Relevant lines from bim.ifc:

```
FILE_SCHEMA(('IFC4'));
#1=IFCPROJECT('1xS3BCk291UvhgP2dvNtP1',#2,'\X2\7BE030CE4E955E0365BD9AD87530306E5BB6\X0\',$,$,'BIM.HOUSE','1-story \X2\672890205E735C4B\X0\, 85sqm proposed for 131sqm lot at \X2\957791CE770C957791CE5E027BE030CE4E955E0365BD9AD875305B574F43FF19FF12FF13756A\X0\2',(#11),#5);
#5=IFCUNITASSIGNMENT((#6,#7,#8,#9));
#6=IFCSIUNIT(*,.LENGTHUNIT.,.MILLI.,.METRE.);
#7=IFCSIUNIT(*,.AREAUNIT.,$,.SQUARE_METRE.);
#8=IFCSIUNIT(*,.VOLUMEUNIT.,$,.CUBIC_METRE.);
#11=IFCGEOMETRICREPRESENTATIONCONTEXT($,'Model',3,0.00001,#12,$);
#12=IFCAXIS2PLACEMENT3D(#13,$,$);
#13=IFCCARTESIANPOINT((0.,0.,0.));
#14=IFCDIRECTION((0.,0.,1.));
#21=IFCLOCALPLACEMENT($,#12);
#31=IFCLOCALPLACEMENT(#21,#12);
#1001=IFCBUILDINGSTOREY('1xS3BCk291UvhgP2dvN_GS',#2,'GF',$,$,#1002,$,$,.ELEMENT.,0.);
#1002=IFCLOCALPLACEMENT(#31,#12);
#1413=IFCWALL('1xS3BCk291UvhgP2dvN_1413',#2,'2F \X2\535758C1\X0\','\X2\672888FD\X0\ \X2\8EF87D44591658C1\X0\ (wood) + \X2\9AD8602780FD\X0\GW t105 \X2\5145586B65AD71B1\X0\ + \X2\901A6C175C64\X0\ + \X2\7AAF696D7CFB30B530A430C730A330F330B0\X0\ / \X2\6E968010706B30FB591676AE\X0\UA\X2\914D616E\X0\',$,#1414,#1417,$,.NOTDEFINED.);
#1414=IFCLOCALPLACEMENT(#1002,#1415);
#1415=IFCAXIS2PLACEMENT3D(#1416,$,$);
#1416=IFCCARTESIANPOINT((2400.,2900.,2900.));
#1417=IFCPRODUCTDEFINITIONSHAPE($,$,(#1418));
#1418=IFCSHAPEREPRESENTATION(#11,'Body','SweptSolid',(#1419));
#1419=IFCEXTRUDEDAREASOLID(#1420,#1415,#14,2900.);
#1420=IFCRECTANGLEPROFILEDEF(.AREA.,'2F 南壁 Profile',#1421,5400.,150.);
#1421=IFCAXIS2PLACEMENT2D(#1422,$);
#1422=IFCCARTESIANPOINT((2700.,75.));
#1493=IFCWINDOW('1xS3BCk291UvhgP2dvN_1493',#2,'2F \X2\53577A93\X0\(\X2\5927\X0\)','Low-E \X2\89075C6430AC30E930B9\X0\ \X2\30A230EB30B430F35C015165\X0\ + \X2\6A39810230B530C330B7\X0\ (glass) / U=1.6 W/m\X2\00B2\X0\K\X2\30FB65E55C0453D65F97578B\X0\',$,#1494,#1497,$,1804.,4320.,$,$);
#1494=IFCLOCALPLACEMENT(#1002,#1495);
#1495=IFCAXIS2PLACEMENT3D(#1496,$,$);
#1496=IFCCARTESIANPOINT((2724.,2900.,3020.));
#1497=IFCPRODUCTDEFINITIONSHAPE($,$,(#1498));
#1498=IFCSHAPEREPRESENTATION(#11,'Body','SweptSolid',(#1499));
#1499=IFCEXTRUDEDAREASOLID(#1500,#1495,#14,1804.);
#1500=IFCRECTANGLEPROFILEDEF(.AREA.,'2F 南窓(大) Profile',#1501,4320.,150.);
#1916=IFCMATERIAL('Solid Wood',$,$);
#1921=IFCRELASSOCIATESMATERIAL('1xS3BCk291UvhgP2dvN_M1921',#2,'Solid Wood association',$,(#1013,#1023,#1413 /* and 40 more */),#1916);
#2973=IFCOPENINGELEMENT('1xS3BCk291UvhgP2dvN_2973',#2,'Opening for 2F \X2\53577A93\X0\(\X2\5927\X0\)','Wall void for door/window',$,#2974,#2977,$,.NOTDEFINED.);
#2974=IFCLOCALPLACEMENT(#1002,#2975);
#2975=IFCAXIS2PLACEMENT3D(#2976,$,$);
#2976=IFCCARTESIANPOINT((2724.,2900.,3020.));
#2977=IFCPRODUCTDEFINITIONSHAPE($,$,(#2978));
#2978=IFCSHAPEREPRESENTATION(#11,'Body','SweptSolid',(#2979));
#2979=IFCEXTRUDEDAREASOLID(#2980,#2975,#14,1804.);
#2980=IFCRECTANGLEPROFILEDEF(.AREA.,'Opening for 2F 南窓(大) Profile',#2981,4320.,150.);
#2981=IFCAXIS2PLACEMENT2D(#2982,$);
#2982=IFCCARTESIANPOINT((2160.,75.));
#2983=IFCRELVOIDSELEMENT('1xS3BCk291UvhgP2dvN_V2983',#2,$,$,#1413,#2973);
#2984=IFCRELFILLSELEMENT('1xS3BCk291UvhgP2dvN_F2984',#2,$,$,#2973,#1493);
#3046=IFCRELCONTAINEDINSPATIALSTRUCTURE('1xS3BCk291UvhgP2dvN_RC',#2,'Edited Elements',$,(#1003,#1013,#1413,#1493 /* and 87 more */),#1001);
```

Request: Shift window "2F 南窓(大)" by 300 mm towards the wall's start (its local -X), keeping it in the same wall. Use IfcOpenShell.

```python
import ifcopenshell
import ifcopenshell.api.geometry
import ifcopenshell.util.placement
import ifcopenshell.util.unit

model = ifcopenshell.open("bim.ifc")
unit_scale = ifcopenshell.util.unit.calculate_unit_scale(model)

window = model.by_guid("1xS3BCk291UvhgP2dvN_1493")
opening = window.FillsVoids[0].RelatingOpeningElement
wall = opening.VoidsElements[0].RelatingBuildingElement

wall_matrix = ifcopenshell.util.placement.get_local_placement(wall.ObjectPlacement)
shift = wall_matrix[:3, 0] * -0.3 / unit_scale
before = ifcopenshell.util.placement.get_local_placement(window.ObjectPlacement)[:3, 3].copy()

# The window is not placed relative to its opening, so move both.
for product in (opening, window):
    matrix = ifcopenshell.util.placement.get_local_placement(product.ObjectPlacement)
    matrix[:3, 3] += shift
    ifcopenshell.api.geometry.edit_object_placement(model, product=product, matrix=matrix, is_si=False)

after = ifcopenshell.util.placement.get_local_placement(window.ObjectPlacement)[:3, 3]
print("window moved by", (after - before).round(3) + 0.0)

model.write("bim_v2.ifc")
```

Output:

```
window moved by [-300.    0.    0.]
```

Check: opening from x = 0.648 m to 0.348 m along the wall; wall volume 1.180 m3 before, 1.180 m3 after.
